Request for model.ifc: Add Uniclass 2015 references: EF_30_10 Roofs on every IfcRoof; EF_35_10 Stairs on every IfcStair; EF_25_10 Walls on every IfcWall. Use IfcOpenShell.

First a look at what the model holds.

```python
import ifcopenshell

model = ifcopenshell.open("model.ifc")
print(model.schema)
print("classifications:", [c.Name for c in model.by_type("IfcClassification")])
for ifc_class in ("IfcDoor", "IfcRoof", "IfcStair", "IfcWall", "IfcWindow"):
    print(ifc_class, len(model.by_type(ifc_class)))
```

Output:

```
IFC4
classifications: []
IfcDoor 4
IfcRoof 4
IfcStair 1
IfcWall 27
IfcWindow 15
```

```python
import ifcopenshell
import ifcopenshell.api.classification

model = ifcopenshell.open("model.ifc")

system = ifcopenshell.api.classification.add_classification(model, classification="Uniclass 2015")

codes = {
    "IfcRoof": ("EF_30_10", "Roofs"),
    "IfcStair": ("EF_35_10", "Stairs"),
    "IfcWall": ("EF_25_10", "Walls"),
}
for ifc_class, (code, name) in codes.items():
    products = model.by_type(ifc_class)
    ifcopenshell.api.classification.add_reference(
        model, products=products, classification=system, identification=code, name=name
    )
    print(code, len(products))

model.write("model_updated.ifc")
```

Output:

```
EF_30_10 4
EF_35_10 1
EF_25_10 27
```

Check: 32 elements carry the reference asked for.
